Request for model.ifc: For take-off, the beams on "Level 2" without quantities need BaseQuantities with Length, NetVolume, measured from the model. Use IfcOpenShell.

First a look at what the model holds.

```python
import ifcopenshell
import ifcopenshell.util.element
import ifcopenshell.util.unit

model = ifcopenshell.open("model.ifc")
print(model.schema)
for unit_type in ("LENGTHUNIT", "AREAUNIT", "VOLUMEUNIT"):
    print(unit_type, ifcopenshell.util.unit.calculate_unit_scale(model, unit_type))
storey = next(s for s in model.by_type("IfcBuildingStorey") if s.Name == "Level 2")
beams = [e for e in ifcopenshell.util.element.get_decomposition(storey) if e.is_a("IfcBeam")]
for e in sorted(beams, key=lambda e: e.id()):
    print(e.id(), e.is_a(), e.Name, list(ifcopenshell.util.element.get_psets(e, qtos_only=True)), sep=" | ")
```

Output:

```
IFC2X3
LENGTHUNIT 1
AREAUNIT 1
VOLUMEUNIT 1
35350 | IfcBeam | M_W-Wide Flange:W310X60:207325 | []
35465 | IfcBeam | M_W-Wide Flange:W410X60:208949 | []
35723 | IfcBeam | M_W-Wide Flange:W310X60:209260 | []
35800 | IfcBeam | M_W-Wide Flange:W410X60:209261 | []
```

```python
import ifcopenshell
import ifcopenshell.api.pset
import ifcopenshell.geom
import ifcopenshell.util.element
import ifcopenshell.util.shape
import ifcopenshell.util.unit

model = ifcopenshell.open("model.ifc")
unit_scale = ifcopenshell.util.unit.calculate_unit_scale(model)
volume_scale = ifcopenshell.util.unit.calculate_unit_scale(model, "VOLUMEUNIT")
settings = ifcopenshell.geom.settings()

storey = next(s for s in model.by_type("IfcBuildingStorey") if s.Name == "Level 2")
beams = [e for e in ifcopenshell.util.element.get_decomposition(storey) if e.is_a("IfcBeam")]

for e in sorted(beams, key=lambda e: e.id()):
    if ifcopenshell.util.element.get_psets(e, qtos_only=True, should_inherit=False):
        continue
    # Geometry comes back in metres, in the element's own axes.
    shape = ifcopenshell.geom.create_shape(settings, e)
    values = {
        "Length": ifcopenshell.util.shape.get_max_xyz(shape.geometry) / unit_scale,
        "NetVolume": ifcopenshell.util.shape.get_volume(shape.geometry) / volume_scale,
    }
    qto = ifcopenshell.api.pset.add_qto(model, product=e, name="BaseQuantities")
    ifcopenshell.api.pset.edit_qto(model, qto=qto, properties=values)
    print(e.id(), {k: round(v, 3) for k, v in values.items()})

model.write("model_updated.ifc")
```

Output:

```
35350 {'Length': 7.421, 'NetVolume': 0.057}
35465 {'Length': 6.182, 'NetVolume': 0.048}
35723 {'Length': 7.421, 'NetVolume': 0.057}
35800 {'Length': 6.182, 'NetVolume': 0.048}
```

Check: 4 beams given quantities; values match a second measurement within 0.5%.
